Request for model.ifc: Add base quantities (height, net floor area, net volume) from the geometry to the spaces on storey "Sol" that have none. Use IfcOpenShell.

First a look at what the model holds.

```python
import ifcopenshell
import ifcopenshell.util.element
import ifcopenshell.util.unit

model = ifcopenshell.open("model.ifc")
print(model.schema)
for unit_type in ("LENGTHUNIT", "AREAUNIT", "VOLUMEUNIT"):
    print(unit_type, ifcopenshell.util.unit.calculate_unit_scale(model, unit_type))
storey = next(s for s in model.by_type("IfcBuildingStorey") if s.Name == "Sol")
spaces = [e for e in ifcopenshell.util.element.get_decomposition(storey) if e.is_a("IfcSpace")]
for e in sorted(spaces, key=lambda e: e.id()):
    print(e.id(), e.is_a(), e.Name, list(ifcopenshell.util.element.get_psets(e, qtos_only=True)), sep=" | ")
```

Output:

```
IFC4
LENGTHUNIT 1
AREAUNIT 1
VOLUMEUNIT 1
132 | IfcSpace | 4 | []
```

```python
import ifcopenshell
import ifcopenshell.api.pset
import ifcopenshell.geom
import ifcopenshell.util.element
import ifcopenshell.util.shape
import ifcopenshell.util.unit

model = ifcopenshell.open("model.ifc")
unit_scale = ifcopenshell.util.unit.calculate_unit_scale(model)
area_scale = ifcopenshell.util.unit.calculate_unit_scale(model, "AREAUNIT")
volume_scale = ifcopenshell.util.unit.calculate_unit_scale(model, "VOLUMEUNIT")
settings = ifcopenshell.geom.settings()

storey = next(s for s in model.by_type("IfcBuildingStorey") if s.Name == "Sol")
spaces = [e for e in ifcopenshell.util.element.get_decomposition(storey) if e.is_a("IfcSpace")]

for e in sorted(spaces, key=lambda e: e.id()):
    if ifcopenshell.util.element.get_psets(e, qtos_only=True, should_inherit=False):
        continue
    # Geometry comes back in metres, in the element's own axes.
    shape = ifcopenshell.geom.create_shape(settings, e)
    values = {
        "Height": ifcopenshell.util.shape.get_z(shape.geometry) / unit_scale,
        "NetFloorArea": ifcopenshell.util.shape.get_footprint_area(shape.geometry) / area_scale,
        "NetVolume": ifcopenshell.util.shape.get_volume(shape.geometry) / volume_scale,
    }
    qto = ifcopenshell.api.pset.add_qto(model, product=e, name="Qto_SpaceBaseQuantities")
    ifcopenshell.api.pset.edit_qto(model, qto=qto, properties=values)
    print(e.id(), {k: round(v, 3) for k, v in values.items()})

model.write("model_v2.ifc")
```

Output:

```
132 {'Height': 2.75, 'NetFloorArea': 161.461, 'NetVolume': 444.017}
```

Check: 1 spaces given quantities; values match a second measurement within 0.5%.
